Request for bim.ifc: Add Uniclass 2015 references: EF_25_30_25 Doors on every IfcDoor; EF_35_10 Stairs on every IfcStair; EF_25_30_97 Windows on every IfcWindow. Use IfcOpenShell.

First a look at what the model holds.

```python
import ifcopenshell

model = ifcopenshell.open("bim.ifc")
print(model.schema)
print("classifications:", [c.Name for c in model.by_type("IfcClassification")])
for ifc_class in ("IfcDoor", "IfcRoof", "IfcStair", "IfcWall", "IfcWindow"):
    print(ifc_class, len(model.by_type(ifc_class)))
```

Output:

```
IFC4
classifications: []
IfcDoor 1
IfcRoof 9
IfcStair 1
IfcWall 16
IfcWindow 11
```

```python
import ifcopenshell
import ifcopenshell.api.classification

model = ifcopenshell.open("bim.ifc")

system = ifcopenshell.api.classification.add_classification(model, classification="Uniclass 2015")

codes = {
    "IfcDoor": ("EF_25_30_25", "Doors"),
    "IfcStair": ("EF_35_10", "Stairs"),
    "IfcWindow": ("EF_25_30_97", "Windows"),
}
for ifc_class, (code, name) in codes.items():
    products = model.by_type(ifc_class)
    ifcopenshell.api.classification.add_reference(
        model, products=products, classification=system, identification=code, name=name
    )
    print(code, len(products))

model.write("bim_rev.ifc")
```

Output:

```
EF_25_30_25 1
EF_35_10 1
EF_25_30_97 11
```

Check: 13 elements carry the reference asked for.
